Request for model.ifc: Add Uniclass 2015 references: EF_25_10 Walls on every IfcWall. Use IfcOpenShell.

First a look at what the model holds.

```python
import ifcopenshell

model = ifcopenshell.open("model.ifc")
print(model.schema)
print("classifications:", [c.Name for c in model.by_type("IfcClassification")])
for ifc_class in ("IfcDoor", "IfcRoof", "IfcStair", "IfcWall", "IfcWindow"):
    print(ifc_class, len(model.by_type(ifc_class)))
```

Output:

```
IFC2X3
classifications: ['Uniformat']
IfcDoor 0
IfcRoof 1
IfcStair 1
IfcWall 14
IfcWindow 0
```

```python
import ifcopenshell
import ifcopenshell.api.classification

model = ifcopenshell.open("model.ifc")

# IFC2X3 requires Source and Edition and has no link from the project to the system.
system = model.create_entity("IfcClassification", Source="NBS", Edition="2015", Name="Uniclass 2015")

codes = {
    "IfcWall": ("EF_25_10", "Walls"),
}
for ifc_class, (code, name) in codes.items():
    products = model.by_type(ifc_class)
    ifcopenshell.api.classification.add_reference(
        model, products=products, classification=system, identification=code, name=name
    )
    print(code, len(products))

model.write("model-out.ifc")
```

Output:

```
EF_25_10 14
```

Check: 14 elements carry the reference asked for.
